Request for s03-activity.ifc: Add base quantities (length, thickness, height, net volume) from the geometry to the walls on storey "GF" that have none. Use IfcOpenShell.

First a look at what the model holds.

```python
import ifcopenshell
import ifcopenshell.util.element
import ifcopenshell.util.unit

model = ifcopenshell.open("s03-activity.ifc")
print(model.schema)
for unit_type in ("LENGTHUNIT", "AREAUNIT", "VOLUMEUNIT"):
    print(unit_type, ifcopenshell.util.unit.calculate_unit_scale(model, unit_type))
storey = next(s for s in model.by_type("IfcBuildingStorey") if s.Name == "GF")
walls = [e for e in ifcopenshell.util.element.get_decomposition(storey) if e.is_a("IfcWall")]
for e in sorted(walls, key=lambda e: e.id()):
    print(e.id(), e.is_a(), e.Name, list(ifcopenshell.util.element.get_psets(e, qtos_only=True)), sep=" | ")
```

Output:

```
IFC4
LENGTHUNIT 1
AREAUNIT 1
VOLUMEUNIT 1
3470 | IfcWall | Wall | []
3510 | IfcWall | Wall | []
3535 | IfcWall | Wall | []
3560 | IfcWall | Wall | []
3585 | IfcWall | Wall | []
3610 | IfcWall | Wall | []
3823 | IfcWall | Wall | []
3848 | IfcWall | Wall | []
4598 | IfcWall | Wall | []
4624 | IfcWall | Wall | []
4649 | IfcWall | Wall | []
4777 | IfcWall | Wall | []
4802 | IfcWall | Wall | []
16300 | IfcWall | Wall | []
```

```python
import ifcopenshell
import ifcopenshell.api.pset
import ifcopenshell.geom
import ifcopenshell.util.element
import ifcopenshell.util.shape
import ifcopenshell.util.unit

model = ifcopenshell.open("s03-activity.ifc")
unit_scale = ifcopenshell.util.unit.calculate_unit_scale(model)
volume_scale = ifcopenshell.util.unit.calculate_unit_scale(model, "VOLUMEUNIT")
settings = ifcopenshell.geom.settings()

storey = next(s for s in model.by_type("IfcBuildingStorey") if s.Name == "GF")
walls = [e for e in ifcopenshell.util.element.get_decomposition(storey) if e.is_a("IfcWall")]

for e in sorted(walls, key=lambda e: e.id()):
    if ifcopenshell.util.element.get_psets(e, qtos_only=True, should_inherit=False):
        continue
    # Geometry comes back in metres, in the element's own axes.
    shape = ifcopenshell.geom.create_shape(settings, e)
    values = {
        "Length": ifcopenshell.util.shape.get_x(shape.geometry) / unit_scale,
        "Width": ifcopenshell.util.shape.get_y(shape.geometry) / unit_scale,
        "Height": ifcopenshell.util.shape.get_z(shape.geometry) / unit_scale,
        "NetVolume": ifcopenshell.util.shape.get_volume(shape.geometry) / volume_scale,
    }
    qto = ifcopenshell.api.pset.add_qto(model, product=e, name="Qto_WallBaseQuantities")
    ifcopenshell.api.pset.edit_qto(model, qto=qto, properties=values)
    print(e.id(), {k: round(v, 3) for k, v in values.items()})

model.write("s03-activity_updated.ifc")
```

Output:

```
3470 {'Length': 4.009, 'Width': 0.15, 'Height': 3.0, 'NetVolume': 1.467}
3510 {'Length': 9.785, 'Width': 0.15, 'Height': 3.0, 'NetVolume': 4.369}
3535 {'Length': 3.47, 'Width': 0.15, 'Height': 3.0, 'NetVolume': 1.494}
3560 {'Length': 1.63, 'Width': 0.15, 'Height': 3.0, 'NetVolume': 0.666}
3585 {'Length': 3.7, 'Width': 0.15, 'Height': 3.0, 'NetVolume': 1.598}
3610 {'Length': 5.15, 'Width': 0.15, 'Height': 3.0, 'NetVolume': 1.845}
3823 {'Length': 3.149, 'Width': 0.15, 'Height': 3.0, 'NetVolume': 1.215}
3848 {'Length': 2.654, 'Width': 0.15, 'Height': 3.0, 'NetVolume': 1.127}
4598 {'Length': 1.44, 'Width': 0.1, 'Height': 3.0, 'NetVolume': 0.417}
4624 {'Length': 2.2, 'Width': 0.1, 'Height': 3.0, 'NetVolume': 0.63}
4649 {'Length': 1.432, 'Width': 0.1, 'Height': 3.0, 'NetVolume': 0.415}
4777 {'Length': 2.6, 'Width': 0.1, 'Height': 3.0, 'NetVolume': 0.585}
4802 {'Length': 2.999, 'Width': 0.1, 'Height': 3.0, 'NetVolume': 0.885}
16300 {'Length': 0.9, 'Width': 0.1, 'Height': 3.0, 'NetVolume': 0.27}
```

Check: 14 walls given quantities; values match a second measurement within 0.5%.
